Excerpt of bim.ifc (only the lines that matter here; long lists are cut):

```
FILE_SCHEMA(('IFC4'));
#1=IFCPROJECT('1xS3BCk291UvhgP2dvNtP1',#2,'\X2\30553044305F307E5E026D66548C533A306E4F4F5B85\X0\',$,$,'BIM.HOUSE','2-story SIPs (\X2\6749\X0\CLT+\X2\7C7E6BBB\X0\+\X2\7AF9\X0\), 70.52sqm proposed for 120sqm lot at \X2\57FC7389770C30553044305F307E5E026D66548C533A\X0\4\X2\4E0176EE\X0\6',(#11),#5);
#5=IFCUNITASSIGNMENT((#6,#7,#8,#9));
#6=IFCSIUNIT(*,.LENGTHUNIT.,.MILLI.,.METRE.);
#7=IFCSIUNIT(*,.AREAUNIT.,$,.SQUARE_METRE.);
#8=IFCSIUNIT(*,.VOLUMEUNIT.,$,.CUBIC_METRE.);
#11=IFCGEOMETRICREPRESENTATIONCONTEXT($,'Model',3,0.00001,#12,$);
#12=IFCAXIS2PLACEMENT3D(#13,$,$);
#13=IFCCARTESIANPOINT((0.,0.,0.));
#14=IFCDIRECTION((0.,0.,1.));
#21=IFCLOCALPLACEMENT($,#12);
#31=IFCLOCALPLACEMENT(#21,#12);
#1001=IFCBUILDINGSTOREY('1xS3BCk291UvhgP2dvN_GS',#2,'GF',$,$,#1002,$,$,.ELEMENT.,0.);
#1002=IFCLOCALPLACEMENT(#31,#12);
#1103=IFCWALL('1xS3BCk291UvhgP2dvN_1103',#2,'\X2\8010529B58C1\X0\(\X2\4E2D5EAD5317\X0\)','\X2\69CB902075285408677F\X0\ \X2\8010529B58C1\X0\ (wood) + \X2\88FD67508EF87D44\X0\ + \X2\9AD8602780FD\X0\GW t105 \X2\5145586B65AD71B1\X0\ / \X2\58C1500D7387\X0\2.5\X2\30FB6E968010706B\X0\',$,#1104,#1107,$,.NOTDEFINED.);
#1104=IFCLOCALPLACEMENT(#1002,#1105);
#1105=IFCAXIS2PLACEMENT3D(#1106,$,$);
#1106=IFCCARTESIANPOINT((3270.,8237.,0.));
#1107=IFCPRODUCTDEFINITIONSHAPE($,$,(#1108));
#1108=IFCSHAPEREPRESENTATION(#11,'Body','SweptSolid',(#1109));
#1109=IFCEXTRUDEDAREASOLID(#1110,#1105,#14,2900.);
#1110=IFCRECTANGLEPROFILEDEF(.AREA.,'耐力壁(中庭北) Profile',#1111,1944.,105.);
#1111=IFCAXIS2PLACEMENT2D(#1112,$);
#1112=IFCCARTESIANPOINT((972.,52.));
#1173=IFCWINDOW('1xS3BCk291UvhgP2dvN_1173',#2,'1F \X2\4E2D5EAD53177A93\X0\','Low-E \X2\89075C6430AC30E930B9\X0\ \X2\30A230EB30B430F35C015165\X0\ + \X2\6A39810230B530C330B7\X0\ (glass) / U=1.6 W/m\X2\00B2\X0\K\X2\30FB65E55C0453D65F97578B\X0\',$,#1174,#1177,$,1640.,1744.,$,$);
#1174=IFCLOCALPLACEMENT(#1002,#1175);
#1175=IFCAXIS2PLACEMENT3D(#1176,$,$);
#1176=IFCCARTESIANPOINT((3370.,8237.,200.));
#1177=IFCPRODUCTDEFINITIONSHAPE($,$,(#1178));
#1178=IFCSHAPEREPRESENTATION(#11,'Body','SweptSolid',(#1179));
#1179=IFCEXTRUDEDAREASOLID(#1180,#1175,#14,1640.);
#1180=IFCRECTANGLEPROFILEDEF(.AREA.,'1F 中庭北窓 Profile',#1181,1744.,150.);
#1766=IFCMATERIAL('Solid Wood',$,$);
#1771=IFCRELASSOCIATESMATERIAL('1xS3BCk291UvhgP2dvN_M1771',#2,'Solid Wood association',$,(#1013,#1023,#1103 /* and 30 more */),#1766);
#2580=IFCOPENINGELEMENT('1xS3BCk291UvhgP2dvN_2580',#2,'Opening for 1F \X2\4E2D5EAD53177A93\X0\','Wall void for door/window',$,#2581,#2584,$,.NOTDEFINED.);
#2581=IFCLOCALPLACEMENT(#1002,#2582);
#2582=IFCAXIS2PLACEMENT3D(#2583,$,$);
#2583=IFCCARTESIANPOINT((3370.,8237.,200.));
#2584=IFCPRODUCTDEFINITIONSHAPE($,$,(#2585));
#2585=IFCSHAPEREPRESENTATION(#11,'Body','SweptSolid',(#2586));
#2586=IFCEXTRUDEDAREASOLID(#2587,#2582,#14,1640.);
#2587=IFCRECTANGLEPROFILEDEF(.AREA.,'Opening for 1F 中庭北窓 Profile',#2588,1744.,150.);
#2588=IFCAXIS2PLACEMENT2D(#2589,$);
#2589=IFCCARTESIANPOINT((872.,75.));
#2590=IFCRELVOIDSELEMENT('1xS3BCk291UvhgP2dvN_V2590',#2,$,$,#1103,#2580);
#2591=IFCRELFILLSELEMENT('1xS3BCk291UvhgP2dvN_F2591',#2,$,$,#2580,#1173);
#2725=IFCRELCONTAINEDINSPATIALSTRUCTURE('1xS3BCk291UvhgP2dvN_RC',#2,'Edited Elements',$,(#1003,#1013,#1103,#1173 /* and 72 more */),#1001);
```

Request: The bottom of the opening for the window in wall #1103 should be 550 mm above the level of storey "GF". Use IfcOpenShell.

```python
import numpy as np
import ifcopenshell
import ifcopenshell.api.geometry
import ifcopenshell.geom
import ifcopenshell.util.element
import ifcopenshell.util.placement
import ifcopenshell.util.shape
import ifcopenshell.util.unit

model = ifcopenshell.open("bim.ifc")
unit_scale = ifcopenshell.util.unit.calculate_unit_scale(model)

window = model.by_id(1173)
opening = window.FillsVoids[0].RelatingOpeningElement
storey = ifcopenshell.util.element.get_container(window, ifc_class="IfcBuildingStorey")
level = ifcopenshell.util.placement.get_local_placement(storey.ObjectPlacement)[2, 3]

# The opening's origin need not be at the sill, so measure its lowest point.
shape = ifcopenshell.geom.create_shape(ifcopenshell.geom.settings(), opening)
bottom = ifcopenshell.util.shape.get_shape_bottom_elevation(shape, shape.geometry) / unit_scale
dz = level + 550.0 - bottom

shift = np.array([0.0, 0.0, dz])
# The window is not placed relative to its opening, so move both.
for product in (opening, window):
    matrix = ifcopenshell.util.placement.get_local_placement(product.ObjectPlacement)
    matrix[:3, 3] += shift
    ifcopenshell.api.geometry.edit_object_placement(model, product=product, matrix=matrix, is_si=False)

print(f"moved by {dz * unit_scale:+.3f} m")

model.write("bim_rev.ifc")
```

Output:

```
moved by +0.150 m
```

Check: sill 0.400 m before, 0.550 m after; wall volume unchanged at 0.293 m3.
